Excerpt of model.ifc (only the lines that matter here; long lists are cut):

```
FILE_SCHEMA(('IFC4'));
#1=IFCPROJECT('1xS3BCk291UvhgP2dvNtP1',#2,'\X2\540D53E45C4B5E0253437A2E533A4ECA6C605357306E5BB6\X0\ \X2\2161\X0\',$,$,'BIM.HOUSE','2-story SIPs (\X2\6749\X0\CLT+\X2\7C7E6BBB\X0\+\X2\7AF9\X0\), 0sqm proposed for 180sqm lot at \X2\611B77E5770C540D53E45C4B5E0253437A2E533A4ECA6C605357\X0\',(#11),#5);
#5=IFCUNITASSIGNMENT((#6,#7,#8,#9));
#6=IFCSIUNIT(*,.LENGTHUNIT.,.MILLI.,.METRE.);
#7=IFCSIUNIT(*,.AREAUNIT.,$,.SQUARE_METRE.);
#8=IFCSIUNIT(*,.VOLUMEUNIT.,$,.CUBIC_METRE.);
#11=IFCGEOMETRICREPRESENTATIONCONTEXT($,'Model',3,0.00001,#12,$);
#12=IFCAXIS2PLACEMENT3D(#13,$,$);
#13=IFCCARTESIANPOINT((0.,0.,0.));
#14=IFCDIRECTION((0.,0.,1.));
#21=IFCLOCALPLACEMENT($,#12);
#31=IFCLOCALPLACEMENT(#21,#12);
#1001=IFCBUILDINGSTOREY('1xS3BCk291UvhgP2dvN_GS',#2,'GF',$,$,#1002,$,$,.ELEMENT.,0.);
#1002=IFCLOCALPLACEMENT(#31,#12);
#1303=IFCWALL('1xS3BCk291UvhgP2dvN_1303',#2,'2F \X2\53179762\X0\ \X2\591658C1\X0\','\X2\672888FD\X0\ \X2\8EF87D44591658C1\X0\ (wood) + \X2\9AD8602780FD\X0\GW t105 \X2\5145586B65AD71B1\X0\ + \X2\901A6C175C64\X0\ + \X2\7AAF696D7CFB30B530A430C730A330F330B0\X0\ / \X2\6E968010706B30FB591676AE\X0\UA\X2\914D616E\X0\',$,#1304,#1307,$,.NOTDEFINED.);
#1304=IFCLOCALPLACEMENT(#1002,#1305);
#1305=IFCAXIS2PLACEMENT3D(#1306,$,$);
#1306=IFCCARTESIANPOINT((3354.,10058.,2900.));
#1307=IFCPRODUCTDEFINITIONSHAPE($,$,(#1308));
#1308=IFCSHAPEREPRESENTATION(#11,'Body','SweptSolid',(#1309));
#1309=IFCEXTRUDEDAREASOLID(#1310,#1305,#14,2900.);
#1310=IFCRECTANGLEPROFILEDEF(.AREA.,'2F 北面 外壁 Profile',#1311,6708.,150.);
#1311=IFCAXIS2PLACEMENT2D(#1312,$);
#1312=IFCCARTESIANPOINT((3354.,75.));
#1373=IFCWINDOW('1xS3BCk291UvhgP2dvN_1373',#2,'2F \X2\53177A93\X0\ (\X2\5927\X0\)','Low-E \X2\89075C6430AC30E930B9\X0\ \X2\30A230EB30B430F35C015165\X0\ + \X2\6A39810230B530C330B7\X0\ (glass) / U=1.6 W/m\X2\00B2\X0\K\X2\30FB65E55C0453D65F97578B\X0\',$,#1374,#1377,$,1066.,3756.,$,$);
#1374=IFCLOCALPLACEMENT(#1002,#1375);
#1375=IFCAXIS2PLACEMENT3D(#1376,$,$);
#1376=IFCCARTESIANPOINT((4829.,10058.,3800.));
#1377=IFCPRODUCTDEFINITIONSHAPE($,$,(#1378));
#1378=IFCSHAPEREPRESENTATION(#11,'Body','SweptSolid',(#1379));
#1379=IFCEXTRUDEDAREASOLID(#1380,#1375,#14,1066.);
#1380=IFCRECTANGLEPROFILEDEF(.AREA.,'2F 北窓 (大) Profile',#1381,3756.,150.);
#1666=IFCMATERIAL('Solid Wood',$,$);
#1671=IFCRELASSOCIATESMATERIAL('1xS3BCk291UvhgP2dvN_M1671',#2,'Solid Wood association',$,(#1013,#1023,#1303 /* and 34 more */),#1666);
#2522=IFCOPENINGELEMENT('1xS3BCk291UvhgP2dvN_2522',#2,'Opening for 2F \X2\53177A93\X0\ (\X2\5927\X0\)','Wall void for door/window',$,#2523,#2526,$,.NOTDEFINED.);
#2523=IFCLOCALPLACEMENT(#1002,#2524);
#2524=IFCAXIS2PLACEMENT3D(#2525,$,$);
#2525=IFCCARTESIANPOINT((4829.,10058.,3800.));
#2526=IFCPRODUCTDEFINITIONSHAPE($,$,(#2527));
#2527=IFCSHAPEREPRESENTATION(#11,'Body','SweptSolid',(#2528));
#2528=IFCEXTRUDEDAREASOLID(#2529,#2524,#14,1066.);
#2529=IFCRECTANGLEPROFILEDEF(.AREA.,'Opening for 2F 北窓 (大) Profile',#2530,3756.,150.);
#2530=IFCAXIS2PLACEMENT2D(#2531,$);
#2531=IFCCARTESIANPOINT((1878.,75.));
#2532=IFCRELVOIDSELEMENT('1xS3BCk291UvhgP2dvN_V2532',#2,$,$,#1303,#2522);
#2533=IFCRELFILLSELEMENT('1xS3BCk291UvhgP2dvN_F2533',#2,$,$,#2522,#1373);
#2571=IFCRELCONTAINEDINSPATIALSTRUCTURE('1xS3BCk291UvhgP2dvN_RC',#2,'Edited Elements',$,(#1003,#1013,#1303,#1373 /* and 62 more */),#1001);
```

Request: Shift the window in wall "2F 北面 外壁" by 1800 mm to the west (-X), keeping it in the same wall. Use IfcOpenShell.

```python
import ifcopenshell
import ifcopenshell.api.geometry
import ifcopenshell.util.placement

model = ifcopenshell.open("model.ifc")

window = model.by_guid("1xS3BCk291UvhgP2dvN_1373")
opening = window.FillsVoids[0].RelatingOpeningElement
wall = opening.VoidsElements[0].RelatingBuildingElement

wall_matrix = ifcopenshell.util.placement.get_local_placement(wall.ObjectPlacement)
shift = wall_matrix[:3, 0] * -1800.0
before = ifcopenshell.util.placement.get_local_placement(window.ObjectPlacement)[:3, 3].copy()

# The window is not placed relative to its opening, so move both.
for product in (opening, window):
    matrix = ifcopenshell.util.placement.get_local_placement(product.ObjectPlacement)
    matrix[:3, 3] += shift
    ifcopenshell.api.geometry.edit_object_placement(model, product=product, matrix=matrix, is_si=False)

after = ifcopenshell.util.placement.get_local_placement(window.ObjectPlacement)[:3, 3]
print("window moved by", (after - before).round(3) + 0.0)

model.write("model_v2.ifc")
```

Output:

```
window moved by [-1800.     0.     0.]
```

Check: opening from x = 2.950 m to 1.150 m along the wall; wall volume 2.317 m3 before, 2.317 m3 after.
